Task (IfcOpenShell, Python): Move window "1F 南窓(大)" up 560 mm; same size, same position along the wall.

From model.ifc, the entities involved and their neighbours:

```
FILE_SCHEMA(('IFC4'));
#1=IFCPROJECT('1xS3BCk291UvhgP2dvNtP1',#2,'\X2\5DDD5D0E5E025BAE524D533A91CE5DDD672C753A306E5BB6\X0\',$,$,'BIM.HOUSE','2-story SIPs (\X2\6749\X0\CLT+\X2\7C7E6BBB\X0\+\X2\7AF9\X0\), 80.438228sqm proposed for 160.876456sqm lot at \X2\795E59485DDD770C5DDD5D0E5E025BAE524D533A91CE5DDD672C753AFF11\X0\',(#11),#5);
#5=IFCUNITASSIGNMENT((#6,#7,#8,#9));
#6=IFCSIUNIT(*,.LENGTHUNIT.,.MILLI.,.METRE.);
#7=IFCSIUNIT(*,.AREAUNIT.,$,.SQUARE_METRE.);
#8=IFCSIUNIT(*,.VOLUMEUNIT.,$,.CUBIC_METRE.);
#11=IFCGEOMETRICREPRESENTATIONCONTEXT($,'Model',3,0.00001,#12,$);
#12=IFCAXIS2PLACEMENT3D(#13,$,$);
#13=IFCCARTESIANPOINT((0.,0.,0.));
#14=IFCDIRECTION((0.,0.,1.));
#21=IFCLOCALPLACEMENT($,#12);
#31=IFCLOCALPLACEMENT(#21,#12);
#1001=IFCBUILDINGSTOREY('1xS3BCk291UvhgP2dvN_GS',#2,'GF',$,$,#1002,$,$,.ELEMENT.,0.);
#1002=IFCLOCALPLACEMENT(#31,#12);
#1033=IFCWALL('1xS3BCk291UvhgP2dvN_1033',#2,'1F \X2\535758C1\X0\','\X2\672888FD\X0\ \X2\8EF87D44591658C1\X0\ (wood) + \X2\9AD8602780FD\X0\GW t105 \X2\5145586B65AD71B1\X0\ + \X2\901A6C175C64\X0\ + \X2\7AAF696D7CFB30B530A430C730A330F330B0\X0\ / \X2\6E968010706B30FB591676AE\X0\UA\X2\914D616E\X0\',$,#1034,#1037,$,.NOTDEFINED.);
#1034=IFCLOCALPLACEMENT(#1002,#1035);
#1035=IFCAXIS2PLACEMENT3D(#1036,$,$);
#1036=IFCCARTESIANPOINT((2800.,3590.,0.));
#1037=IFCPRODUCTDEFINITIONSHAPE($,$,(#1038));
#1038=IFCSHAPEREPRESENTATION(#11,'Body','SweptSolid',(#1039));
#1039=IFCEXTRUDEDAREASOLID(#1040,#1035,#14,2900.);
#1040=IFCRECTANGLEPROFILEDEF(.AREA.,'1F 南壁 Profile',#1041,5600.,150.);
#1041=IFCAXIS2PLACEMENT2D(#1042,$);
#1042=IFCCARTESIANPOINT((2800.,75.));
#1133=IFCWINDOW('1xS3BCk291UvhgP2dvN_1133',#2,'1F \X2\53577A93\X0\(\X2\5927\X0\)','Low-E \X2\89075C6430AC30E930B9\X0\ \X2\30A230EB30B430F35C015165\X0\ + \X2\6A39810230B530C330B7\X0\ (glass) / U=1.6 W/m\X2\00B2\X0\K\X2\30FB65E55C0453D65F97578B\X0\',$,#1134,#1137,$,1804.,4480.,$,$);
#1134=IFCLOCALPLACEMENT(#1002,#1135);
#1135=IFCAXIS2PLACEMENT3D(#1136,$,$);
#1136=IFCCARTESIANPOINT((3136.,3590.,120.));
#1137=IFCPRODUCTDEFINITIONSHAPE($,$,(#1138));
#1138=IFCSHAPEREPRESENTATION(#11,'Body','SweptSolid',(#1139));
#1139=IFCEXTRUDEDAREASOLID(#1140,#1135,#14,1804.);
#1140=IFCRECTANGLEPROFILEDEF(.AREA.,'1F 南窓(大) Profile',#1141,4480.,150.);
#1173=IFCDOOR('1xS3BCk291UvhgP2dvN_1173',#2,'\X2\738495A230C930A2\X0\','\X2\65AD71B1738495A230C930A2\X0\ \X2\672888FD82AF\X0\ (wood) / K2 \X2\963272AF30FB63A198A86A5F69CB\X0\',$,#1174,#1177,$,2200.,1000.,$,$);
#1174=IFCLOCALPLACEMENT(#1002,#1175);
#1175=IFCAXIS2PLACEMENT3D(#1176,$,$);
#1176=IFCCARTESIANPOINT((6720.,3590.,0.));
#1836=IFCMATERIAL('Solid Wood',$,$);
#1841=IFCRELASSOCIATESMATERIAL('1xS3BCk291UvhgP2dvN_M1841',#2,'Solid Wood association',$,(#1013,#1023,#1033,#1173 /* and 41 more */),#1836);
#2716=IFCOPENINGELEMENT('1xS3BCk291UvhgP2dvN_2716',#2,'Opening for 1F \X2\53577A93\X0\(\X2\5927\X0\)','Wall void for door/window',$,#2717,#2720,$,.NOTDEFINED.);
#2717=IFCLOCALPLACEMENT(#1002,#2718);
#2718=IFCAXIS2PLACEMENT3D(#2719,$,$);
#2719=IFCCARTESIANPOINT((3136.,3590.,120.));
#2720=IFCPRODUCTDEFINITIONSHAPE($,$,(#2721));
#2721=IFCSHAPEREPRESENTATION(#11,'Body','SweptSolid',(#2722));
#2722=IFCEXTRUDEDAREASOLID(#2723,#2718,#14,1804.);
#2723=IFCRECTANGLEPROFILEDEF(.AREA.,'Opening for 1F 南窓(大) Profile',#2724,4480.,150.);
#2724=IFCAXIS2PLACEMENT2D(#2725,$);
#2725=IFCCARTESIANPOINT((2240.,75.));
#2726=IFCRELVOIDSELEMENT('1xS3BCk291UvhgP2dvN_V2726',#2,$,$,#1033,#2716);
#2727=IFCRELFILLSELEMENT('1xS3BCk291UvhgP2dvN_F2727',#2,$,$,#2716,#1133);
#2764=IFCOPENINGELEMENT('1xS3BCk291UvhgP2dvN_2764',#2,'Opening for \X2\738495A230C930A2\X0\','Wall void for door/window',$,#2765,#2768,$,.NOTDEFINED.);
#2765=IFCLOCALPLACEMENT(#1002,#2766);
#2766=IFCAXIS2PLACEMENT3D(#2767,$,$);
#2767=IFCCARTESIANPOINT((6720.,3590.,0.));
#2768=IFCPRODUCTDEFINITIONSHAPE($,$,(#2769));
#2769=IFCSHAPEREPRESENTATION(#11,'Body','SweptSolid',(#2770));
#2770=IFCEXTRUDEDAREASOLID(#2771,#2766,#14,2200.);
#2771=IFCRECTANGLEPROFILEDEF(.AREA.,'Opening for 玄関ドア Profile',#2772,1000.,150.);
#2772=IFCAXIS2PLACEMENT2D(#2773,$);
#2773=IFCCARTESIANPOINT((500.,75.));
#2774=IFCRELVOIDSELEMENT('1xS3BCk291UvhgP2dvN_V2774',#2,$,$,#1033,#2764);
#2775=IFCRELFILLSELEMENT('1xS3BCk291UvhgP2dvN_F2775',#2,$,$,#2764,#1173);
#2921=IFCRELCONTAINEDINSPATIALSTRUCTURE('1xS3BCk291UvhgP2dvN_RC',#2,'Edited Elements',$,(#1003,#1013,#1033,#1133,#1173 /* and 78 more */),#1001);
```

```python
import numpy as np
import ifcopenshell
import ifcopenshell.api.geometry
import ifcopenshell.util.placement
import ifcopenshell.util.unit

model = ifcopenshell.open("model.ifc")
unit_scale = ifcopenshell.util.unit.calculate_unit_scale(model)

window = model.by_guid("1xS3BCk291UvhgP2dvN_1133")
opening = window.FillsVoids[0].RelatingOpeningElement
dz = 560.0

shift = np.array([0.0, 0.0, dz])
# The window is not placed relative to its opening, so move both.
for product in (opening, window):
    matrix = ifcopenshell.util.placement.get_local_placement(product.ObjectPlacement)
    matrix[:3, 3] += shift
    ifcopenshell.api.geometry.edit_object_placement(model, product=product, matrix=matrix, is_si=False)

print(f"moved by {dz * unit_scale:+.3f} m")

model.write("model_edited.ifc")
```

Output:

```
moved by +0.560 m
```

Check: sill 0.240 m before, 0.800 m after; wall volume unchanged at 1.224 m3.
